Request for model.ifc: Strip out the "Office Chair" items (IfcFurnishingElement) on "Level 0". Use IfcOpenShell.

First a look at what the model holds.

```python
import ifcopenshell
import ifcopenshell.util.element

model = ifcopenshell.open("model.ifc")
print(model.schema)
storey = next(s for s in model.by_type("IfcBuildingStorey") if s.Name == "Level 0")
furniture = [e for e in ifcopenshell.util.element.get_decomposition(storey) if e.is_a("IfcFurnishingElement")]
seen = {}
for e in furniture:
    element_type = ifcopenshell.util.element.get_type(e)
    name = element_type.Name if element_type not in (None, e) else None
    seen[name] = seen.get(name, 0) + 1
for name, count in sorted(seen.items(), key=str):
    print(count, "x", name)
```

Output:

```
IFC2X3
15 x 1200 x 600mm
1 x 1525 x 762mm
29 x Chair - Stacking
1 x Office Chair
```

```python
import ifcopenshell
import ifcopenshell.api.root
import ifcopenshell.util.element

model = ifcopenshell.open("model.ifc")

storey = next(s for s in model.by_type("IfcBuildingStorey") if s.Name == "Level 0")
furniture = [e for e in ifcopenshell.util.element.get_decomposition(storey) if e.is_a("IfcFurnishingElement")]
targets = [e for e in furniture if (t := ifcopenshell.util.element.get_type(e)) not in (None, e) and t.Name == "Office Chair"]

for e in targets:
    ifcopenshell.api.root.remove_product(model, product=e)
print(len(targets), "removed")

model.write("model_edited.ifc")
```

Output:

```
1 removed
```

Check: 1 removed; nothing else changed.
